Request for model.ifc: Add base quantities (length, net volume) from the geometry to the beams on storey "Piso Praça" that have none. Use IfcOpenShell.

First a look at what the model holds.

```python
import ifcopenshell
import ifcopenshell.util.element
import ifcopenshell.util.unit

model = ifcopenshell.open("model.ifc")
print(model.schema)
for unit_type in ("LENGTHUNIT", "AREAUNIT", "VOLUMEUNIT"):
    print(unit_type, ifcopenshell.util.unit.calculate_unit_scale(model, unit_type))
storey = next(s for s in model.by_type("IfcBuildingStorey") if s.Name == "Piso Praça")
beams = [e for e in ifcopenshell.util.element.get_decomposition(storey) if e.is_a("IfcBeam")]
for e in sorted(beams, key=lambda e: e.id()):
    print(e.id(), e.is_a(), e.Name, list(ifcopenshell.util.element.get_psets(e, qtos_only=True)), sep=" | ")
```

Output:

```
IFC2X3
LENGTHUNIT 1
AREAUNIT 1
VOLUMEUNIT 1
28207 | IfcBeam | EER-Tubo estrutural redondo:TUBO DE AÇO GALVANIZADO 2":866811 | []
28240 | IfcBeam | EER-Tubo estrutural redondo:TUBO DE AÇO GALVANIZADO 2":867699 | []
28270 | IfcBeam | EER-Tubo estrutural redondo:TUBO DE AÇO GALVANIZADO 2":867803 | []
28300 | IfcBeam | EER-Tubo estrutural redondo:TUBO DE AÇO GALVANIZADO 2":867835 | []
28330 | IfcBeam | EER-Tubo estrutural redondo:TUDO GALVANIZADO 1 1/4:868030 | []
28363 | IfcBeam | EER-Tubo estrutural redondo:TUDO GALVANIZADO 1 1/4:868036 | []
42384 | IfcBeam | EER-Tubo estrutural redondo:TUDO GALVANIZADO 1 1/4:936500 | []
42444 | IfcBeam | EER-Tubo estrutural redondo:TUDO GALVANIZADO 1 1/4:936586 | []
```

```python
import ifcopenshell
import ifcopenshell.api.pset
import ifcopenshell.geom
import ifcopenshell.util.element
import ifcopenshell.util.shape
import ifcopenshell.util.unit

model = ifcopenshell.open("model.ifc")
unit_scale = ifcopenshell.util.unit.calculate_unit_scale(model)
volume_scale = ifcopenshell.util.unit.calculate_unit_scale(model, "VOLUMEUNIT")
settings = ifcopenshell.geom.settings()

storey = next(s for s in model.by_type("IfcBuildingStorey") if s.Name == "Piso Praça")
beams = [e for e in ifcopenshell.util.element.get_decomposition(storey) if e.is_a("IfcBeam")]

for e in sorted(beams, key=lambda e: e.id()):
    if ifcopenshell.util.element.get_psets(e, qtos_only=True, should_inherit=False):
        continue
    # Geometry comes back in metres, in the element's own axes.
    shape = ifcopenshell.geom.create_shape(settings, e)
    values = {
        "Length": ifcopenshell.util.shape.get_max_xyz(shape.geometry) / unit_scale,
        "NetVolume": ifcopenshell.util.shape.get_volume(shape.geometry) / volume_scale,
    }
    qto = ifcopenshell.api.pset.add_qto(model, product=e, name="BaseQuantities")
    ifcopenshell.api.pset.edit_qto(model, qto=qto, properties=values)
    print(e.id(), {k: round(v, 3) for k, v in values.items()})

model.write("model_updated.ifc")
```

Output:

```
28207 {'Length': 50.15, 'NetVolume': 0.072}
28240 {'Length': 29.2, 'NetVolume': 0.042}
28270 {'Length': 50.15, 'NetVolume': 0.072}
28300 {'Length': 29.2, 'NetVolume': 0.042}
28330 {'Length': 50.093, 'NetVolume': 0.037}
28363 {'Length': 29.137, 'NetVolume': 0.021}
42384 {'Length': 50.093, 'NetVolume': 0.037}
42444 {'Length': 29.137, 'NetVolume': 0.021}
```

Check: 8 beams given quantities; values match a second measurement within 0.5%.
